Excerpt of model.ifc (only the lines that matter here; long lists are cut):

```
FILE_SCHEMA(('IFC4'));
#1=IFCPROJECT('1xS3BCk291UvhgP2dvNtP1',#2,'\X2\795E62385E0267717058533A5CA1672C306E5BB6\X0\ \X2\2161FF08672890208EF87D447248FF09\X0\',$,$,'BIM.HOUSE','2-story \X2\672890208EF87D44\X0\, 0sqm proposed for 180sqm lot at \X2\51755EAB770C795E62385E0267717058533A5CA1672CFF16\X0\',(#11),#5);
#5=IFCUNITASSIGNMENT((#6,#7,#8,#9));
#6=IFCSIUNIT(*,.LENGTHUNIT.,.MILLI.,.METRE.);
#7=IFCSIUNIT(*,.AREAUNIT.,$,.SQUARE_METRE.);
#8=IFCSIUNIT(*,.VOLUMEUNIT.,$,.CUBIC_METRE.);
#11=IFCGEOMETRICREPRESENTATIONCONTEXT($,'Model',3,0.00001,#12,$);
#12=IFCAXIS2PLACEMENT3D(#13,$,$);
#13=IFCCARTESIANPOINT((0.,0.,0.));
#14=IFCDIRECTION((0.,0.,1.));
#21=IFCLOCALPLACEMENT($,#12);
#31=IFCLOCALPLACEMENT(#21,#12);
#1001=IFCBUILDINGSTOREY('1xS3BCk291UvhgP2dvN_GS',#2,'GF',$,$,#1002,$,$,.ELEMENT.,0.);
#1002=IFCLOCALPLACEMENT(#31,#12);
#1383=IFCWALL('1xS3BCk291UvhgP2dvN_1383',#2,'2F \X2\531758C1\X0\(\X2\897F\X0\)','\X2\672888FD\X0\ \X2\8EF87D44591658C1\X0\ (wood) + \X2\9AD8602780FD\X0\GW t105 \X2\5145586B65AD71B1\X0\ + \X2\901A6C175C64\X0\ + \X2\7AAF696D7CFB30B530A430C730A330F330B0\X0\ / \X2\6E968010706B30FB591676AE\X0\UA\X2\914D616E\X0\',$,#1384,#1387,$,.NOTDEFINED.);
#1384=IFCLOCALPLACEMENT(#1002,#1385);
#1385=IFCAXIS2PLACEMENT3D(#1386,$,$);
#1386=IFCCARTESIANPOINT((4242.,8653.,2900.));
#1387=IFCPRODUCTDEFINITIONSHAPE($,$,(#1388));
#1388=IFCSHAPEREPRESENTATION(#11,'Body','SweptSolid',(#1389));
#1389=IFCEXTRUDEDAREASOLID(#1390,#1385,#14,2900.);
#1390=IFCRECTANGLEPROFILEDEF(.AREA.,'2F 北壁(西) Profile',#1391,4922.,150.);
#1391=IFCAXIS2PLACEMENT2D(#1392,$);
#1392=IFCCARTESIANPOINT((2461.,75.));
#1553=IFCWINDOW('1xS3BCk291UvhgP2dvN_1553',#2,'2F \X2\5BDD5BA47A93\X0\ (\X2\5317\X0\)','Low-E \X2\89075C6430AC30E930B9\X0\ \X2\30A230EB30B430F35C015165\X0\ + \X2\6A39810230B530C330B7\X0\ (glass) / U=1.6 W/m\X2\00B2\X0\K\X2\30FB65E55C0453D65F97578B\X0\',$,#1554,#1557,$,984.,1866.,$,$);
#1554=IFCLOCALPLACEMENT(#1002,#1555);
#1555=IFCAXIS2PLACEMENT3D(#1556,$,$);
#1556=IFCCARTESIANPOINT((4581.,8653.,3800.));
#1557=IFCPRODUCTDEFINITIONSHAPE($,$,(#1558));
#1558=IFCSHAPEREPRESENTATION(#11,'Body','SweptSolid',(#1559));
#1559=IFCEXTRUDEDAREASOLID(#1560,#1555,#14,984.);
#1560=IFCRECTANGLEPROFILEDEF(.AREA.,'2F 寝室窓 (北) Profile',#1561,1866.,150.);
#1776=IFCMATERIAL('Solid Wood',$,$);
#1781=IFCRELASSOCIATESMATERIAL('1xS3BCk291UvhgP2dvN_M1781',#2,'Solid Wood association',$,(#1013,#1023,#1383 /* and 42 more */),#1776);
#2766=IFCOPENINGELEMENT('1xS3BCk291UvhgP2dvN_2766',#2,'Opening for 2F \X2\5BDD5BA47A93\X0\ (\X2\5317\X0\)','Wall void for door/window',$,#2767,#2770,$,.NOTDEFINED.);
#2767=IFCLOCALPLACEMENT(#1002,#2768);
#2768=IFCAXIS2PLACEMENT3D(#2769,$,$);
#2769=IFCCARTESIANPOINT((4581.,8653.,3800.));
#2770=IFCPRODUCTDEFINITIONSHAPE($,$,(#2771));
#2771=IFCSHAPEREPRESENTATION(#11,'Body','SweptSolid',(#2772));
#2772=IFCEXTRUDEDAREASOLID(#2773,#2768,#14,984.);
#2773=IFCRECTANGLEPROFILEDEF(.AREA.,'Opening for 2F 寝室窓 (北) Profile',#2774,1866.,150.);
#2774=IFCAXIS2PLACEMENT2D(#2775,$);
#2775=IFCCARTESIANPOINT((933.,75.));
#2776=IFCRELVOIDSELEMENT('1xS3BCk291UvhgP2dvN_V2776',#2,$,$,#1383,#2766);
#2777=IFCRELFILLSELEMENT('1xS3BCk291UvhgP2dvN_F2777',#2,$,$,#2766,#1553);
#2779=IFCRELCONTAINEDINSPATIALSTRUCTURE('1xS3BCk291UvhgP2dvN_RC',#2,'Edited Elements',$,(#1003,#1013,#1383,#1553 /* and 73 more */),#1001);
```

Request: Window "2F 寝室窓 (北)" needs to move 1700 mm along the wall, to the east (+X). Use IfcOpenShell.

```python
import ifcopenshell
import ifcopenshell.api.geometry
import ifcopenshell.util.placement
import ifcopenshell.util.unit

model = ifcopenshell.open("model.ifc")
unit_scale = ifcopenshell.util.unit.calculate_unit_scale(model)

window = model.by_guid("1xS3BCk291UvhgP2dvN_1553")
opening = window.FillsVoids[0].RelatingOpeningElement
wall = opening.VoidsElements[0].RelatingBuildingElement

wall_matrix = ifcopenshell.util.placement.get_local_placement(wall.ObjectPlacement)
shift = wall_matrix[:3, 0] * 1.7 / unit_scale
before = ifcopenshell.util.placement.get_local_placement(window.ObjectPlacement)[:3, 3].copy()

# The window is not placed relative to its opening, so move both.
for product in (opening, window):
    matrix = ifcopenshell.util.placement.get_local_placement(product.ObjectPlacement)
    matrix[:3, 3] += shift
    ifcopenshell.api.geometry.edit_object_placement(model, product=product, matrix=matrix, is_si=False)

after = ifcopenshell.util.placement.get_local_placement(window.ObjectPlacement)[:3, 3]
print("window moved by", (after - before).round(3) + 0.0)

model.write("model-out.ifc")
```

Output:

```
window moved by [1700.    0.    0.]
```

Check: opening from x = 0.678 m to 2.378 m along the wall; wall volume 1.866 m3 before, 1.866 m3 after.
